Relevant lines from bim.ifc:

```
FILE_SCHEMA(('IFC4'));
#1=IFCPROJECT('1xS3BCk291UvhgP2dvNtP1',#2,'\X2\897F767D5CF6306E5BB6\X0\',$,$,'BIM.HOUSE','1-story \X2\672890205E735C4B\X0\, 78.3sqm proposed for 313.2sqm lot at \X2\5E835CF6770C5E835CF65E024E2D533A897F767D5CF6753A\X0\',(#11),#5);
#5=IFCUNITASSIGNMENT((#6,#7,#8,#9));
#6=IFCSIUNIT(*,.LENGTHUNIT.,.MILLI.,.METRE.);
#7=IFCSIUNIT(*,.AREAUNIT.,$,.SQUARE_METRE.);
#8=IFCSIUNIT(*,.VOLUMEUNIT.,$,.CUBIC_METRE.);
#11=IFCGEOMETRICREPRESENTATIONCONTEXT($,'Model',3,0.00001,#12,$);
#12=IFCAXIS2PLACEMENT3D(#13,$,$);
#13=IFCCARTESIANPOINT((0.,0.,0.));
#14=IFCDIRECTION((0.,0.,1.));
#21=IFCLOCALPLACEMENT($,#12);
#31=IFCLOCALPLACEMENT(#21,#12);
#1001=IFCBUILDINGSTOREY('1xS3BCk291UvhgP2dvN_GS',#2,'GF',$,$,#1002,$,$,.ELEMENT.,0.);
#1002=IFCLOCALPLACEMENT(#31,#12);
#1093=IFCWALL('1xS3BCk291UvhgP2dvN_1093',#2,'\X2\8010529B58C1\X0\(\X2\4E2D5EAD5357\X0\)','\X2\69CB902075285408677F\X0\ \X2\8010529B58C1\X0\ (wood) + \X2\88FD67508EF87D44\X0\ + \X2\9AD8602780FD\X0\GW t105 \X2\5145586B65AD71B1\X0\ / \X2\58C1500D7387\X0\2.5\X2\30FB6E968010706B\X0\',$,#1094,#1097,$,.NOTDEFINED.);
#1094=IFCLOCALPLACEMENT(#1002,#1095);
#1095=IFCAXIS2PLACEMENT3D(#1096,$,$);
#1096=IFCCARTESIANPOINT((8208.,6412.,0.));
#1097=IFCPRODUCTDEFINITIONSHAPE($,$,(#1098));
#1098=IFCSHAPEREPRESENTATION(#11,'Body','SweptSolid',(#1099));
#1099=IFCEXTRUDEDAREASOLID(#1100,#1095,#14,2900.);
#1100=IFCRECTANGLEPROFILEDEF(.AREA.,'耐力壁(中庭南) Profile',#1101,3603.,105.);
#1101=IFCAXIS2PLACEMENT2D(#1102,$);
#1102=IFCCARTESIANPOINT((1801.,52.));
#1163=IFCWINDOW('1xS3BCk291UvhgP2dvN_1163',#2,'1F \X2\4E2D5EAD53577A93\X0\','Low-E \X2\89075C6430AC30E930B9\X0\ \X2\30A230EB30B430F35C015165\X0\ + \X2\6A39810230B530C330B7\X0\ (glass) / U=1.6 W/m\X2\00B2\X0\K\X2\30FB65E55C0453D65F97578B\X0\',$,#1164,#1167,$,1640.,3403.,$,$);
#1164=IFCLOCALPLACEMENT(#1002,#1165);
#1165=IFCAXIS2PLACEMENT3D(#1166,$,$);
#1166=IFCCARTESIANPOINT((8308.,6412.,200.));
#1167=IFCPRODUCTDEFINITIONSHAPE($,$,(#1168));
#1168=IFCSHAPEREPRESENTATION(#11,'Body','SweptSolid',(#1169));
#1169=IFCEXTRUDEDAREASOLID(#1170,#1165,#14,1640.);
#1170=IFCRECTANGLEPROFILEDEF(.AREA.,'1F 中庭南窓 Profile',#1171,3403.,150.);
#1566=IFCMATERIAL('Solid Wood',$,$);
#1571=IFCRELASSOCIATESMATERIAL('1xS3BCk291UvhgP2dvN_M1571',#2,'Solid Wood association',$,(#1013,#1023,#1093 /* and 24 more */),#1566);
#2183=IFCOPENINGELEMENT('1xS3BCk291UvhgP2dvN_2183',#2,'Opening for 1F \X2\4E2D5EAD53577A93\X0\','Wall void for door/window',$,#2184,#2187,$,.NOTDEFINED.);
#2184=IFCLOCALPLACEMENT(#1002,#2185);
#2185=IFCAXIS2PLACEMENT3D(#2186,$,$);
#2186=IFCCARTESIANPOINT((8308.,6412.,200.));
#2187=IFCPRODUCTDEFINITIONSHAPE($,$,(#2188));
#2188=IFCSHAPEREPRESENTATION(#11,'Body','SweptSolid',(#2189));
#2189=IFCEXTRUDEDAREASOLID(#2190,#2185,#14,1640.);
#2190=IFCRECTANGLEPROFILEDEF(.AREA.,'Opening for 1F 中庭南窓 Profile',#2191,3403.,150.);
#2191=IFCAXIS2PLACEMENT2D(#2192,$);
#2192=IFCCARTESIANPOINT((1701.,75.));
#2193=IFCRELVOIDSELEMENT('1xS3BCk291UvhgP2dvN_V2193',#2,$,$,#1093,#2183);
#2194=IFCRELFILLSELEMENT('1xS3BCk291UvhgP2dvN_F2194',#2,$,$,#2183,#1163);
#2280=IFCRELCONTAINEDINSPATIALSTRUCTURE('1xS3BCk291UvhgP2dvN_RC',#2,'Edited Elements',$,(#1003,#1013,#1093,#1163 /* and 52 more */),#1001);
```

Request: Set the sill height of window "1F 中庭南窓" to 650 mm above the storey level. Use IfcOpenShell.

```python
import numpy as np
import ifcopenshell
import ifcopenshell.api.geometry
import ifcopenshell.geom
import ifcopenshell.util.element
import ifcopenshell.util.placement
import ifcopenshell.util.shape
import ifcopenshell.util.unit

model = ifcopenshell.open("bim.ifc")
unit_scale = ifcopenshell.util.unit.calculate_unit_scale(model)

window = model.by_guid("1xS3BCk291UvhgP2dvN_1163")
opening = window.FillsVoids[0].RelatingOpeningElement
storey = ifcopenshell.util.element.get_container(window, ifc_class="IfcBuildingStorey")
level = ifcopenshell.util.placement.get_local_placement(storey.ObjectPlacement)[2, 3]

# The opening's origin need not be at the sill, so measure its lowest point.
shape = ifcopenshell.geom.create_shape(ifcopenshell.geom.settings(), opening)
bottom = ifcopenshell.util.shape.get_shape_bottom_elevation(shape, shape.geometry) / unit_scale
dz = level + 650.0 - bottom

shift = np.array([0.0, 0.0, dz])
# The window is not placed relative to its opening, so move both.
for product in (opening, window):
    matrix = ifcopenshell.util.placement.get_local_placement(product.ObjectPlacement)
    matrix[:3, 3] += shift
    ifcopenshell.api.geometry.edit_object_placement(model, product=product, matrix=matrix, is_si=False)

print(f"moved by {dz * unit_scale:+.3f} m")

model.write("bim_rev.ifc")
```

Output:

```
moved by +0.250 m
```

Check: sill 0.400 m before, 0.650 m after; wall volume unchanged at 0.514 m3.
